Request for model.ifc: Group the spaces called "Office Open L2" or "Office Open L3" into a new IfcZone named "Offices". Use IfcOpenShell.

First a look at what the model holds.

```python
import ifcopenshell

model = ifcopenshell.open("model.ifc")
print(model.schema)
seen = {}
for space in model.by_type("IfcSpace"):
    seen[space.Name] = seen.get(space.Name, 0) + 1
for name, count in sorted(seen.items(), key=str):
    print(count, "x", name)
print("zones:", [z.Name for z in model.by_type("IfcZone")][:20])
```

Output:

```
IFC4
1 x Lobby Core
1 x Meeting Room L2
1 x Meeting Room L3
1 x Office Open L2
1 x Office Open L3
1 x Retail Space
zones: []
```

```python
import ifcopenshell
import ifcopenshell.api.group
import ifcopenshell.api.root

model = ifcopenshell.open("model.ifc")

names = {"Office Open L2", "Office Open L3"}
spaces = [s for s in model.by_type("IfcSpace") if s.Name in names]

zone = ifcopenshell.api.root.create_entity(model, ifc_class="IfcZone", name="Offices")
ifcopenshell.api.group.assign_group(model, products=spaces, group=zone)
print(len(spaces), "spaces in", zone.Name)

model.write("model_edited.ifc")
```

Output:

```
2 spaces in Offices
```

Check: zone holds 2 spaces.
